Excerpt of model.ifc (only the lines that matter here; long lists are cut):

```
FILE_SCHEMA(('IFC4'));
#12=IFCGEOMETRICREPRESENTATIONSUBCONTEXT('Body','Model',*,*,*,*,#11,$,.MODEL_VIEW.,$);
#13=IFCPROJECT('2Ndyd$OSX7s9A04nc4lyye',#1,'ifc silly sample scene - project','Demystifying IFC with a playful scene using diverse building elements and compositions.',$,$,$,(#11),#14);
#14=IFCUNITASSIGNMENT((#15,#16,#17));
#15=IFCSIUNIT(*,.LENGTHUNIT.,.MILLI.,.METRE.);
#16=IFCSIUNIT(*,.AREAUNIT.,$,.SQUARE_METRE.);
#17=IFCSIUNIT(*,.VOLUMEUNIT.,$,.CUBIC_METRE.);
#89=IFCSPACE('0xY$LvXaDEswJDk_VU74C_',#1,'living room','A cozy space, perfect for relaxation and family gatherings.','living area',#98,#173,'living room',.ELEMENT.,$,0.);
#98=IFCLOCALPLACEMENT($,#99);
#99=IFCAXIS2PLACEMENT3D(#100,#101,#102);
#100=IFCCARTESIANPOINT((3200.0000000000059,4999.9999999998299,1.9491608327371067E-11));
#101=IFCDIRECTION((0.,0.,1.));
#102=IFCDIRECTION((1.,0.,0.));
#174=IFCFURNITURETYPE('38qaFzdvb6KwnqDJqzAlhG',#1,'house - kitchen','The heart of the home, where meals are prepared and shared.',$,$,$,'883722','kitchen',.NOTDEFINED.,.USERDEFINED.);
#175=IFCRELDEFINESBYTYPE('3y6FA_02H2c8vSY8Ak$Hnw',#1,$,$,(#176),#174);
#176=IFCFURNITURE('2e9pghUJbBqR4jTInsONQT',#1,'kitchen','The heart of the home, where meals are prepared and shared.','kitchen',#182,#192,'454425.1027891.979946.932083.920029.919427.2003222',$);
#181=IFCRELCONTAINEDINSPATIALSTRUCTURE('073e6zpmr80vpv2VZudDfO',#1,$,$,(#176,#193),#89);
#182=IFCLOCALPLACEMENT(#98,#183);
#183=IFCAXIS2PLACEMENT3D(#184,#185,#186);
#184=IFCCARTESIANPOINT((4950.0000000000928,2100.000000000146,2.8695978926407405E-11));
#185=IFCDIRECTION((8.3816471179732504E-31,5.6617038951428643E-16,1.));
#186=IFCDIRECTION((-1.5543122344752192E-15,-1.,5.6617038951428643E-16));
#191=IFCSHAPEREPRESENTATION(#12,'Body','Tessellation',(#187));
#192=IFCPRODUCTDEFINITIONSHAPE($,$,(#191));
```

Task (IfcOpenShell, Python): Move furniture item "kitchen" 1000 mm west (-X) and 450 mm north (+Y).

```python
import ifcopenshell
import ifcopenshell.api.geometry
import ifcopenshell.util.placement
import ifcopenshell.util.unit

model = ifcopenshell.open("model.ifc")
unit_scale = ifcopenshell.util.unit.calculate_unit_scale(model)

item = model.by_id(176)
matrix = ifcopenshell.util.placement.get_local_placement(item.ObjectPlacement)
matrix[0, 3] -= 1 / unit_scale
matrix[1, 3] += 0.45 / unit_scale
ifcopenshell.api.geometry.edit_object_placement(model, product=item, matrix=matrix, is_si=False)

print(ifcopenshell.util.placement.get_local_placement(item.ObjectPlacement).round(3) + 0.0)

model.write("model_updated.ifc")
```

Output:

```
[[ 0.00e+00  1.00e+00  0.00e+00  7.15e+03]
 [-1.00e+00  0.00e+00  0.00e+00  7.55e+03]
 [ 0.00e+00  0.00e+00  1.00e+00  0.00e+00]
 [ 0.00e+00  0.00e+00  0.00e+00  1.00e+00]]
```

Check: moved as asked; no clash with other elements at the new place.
